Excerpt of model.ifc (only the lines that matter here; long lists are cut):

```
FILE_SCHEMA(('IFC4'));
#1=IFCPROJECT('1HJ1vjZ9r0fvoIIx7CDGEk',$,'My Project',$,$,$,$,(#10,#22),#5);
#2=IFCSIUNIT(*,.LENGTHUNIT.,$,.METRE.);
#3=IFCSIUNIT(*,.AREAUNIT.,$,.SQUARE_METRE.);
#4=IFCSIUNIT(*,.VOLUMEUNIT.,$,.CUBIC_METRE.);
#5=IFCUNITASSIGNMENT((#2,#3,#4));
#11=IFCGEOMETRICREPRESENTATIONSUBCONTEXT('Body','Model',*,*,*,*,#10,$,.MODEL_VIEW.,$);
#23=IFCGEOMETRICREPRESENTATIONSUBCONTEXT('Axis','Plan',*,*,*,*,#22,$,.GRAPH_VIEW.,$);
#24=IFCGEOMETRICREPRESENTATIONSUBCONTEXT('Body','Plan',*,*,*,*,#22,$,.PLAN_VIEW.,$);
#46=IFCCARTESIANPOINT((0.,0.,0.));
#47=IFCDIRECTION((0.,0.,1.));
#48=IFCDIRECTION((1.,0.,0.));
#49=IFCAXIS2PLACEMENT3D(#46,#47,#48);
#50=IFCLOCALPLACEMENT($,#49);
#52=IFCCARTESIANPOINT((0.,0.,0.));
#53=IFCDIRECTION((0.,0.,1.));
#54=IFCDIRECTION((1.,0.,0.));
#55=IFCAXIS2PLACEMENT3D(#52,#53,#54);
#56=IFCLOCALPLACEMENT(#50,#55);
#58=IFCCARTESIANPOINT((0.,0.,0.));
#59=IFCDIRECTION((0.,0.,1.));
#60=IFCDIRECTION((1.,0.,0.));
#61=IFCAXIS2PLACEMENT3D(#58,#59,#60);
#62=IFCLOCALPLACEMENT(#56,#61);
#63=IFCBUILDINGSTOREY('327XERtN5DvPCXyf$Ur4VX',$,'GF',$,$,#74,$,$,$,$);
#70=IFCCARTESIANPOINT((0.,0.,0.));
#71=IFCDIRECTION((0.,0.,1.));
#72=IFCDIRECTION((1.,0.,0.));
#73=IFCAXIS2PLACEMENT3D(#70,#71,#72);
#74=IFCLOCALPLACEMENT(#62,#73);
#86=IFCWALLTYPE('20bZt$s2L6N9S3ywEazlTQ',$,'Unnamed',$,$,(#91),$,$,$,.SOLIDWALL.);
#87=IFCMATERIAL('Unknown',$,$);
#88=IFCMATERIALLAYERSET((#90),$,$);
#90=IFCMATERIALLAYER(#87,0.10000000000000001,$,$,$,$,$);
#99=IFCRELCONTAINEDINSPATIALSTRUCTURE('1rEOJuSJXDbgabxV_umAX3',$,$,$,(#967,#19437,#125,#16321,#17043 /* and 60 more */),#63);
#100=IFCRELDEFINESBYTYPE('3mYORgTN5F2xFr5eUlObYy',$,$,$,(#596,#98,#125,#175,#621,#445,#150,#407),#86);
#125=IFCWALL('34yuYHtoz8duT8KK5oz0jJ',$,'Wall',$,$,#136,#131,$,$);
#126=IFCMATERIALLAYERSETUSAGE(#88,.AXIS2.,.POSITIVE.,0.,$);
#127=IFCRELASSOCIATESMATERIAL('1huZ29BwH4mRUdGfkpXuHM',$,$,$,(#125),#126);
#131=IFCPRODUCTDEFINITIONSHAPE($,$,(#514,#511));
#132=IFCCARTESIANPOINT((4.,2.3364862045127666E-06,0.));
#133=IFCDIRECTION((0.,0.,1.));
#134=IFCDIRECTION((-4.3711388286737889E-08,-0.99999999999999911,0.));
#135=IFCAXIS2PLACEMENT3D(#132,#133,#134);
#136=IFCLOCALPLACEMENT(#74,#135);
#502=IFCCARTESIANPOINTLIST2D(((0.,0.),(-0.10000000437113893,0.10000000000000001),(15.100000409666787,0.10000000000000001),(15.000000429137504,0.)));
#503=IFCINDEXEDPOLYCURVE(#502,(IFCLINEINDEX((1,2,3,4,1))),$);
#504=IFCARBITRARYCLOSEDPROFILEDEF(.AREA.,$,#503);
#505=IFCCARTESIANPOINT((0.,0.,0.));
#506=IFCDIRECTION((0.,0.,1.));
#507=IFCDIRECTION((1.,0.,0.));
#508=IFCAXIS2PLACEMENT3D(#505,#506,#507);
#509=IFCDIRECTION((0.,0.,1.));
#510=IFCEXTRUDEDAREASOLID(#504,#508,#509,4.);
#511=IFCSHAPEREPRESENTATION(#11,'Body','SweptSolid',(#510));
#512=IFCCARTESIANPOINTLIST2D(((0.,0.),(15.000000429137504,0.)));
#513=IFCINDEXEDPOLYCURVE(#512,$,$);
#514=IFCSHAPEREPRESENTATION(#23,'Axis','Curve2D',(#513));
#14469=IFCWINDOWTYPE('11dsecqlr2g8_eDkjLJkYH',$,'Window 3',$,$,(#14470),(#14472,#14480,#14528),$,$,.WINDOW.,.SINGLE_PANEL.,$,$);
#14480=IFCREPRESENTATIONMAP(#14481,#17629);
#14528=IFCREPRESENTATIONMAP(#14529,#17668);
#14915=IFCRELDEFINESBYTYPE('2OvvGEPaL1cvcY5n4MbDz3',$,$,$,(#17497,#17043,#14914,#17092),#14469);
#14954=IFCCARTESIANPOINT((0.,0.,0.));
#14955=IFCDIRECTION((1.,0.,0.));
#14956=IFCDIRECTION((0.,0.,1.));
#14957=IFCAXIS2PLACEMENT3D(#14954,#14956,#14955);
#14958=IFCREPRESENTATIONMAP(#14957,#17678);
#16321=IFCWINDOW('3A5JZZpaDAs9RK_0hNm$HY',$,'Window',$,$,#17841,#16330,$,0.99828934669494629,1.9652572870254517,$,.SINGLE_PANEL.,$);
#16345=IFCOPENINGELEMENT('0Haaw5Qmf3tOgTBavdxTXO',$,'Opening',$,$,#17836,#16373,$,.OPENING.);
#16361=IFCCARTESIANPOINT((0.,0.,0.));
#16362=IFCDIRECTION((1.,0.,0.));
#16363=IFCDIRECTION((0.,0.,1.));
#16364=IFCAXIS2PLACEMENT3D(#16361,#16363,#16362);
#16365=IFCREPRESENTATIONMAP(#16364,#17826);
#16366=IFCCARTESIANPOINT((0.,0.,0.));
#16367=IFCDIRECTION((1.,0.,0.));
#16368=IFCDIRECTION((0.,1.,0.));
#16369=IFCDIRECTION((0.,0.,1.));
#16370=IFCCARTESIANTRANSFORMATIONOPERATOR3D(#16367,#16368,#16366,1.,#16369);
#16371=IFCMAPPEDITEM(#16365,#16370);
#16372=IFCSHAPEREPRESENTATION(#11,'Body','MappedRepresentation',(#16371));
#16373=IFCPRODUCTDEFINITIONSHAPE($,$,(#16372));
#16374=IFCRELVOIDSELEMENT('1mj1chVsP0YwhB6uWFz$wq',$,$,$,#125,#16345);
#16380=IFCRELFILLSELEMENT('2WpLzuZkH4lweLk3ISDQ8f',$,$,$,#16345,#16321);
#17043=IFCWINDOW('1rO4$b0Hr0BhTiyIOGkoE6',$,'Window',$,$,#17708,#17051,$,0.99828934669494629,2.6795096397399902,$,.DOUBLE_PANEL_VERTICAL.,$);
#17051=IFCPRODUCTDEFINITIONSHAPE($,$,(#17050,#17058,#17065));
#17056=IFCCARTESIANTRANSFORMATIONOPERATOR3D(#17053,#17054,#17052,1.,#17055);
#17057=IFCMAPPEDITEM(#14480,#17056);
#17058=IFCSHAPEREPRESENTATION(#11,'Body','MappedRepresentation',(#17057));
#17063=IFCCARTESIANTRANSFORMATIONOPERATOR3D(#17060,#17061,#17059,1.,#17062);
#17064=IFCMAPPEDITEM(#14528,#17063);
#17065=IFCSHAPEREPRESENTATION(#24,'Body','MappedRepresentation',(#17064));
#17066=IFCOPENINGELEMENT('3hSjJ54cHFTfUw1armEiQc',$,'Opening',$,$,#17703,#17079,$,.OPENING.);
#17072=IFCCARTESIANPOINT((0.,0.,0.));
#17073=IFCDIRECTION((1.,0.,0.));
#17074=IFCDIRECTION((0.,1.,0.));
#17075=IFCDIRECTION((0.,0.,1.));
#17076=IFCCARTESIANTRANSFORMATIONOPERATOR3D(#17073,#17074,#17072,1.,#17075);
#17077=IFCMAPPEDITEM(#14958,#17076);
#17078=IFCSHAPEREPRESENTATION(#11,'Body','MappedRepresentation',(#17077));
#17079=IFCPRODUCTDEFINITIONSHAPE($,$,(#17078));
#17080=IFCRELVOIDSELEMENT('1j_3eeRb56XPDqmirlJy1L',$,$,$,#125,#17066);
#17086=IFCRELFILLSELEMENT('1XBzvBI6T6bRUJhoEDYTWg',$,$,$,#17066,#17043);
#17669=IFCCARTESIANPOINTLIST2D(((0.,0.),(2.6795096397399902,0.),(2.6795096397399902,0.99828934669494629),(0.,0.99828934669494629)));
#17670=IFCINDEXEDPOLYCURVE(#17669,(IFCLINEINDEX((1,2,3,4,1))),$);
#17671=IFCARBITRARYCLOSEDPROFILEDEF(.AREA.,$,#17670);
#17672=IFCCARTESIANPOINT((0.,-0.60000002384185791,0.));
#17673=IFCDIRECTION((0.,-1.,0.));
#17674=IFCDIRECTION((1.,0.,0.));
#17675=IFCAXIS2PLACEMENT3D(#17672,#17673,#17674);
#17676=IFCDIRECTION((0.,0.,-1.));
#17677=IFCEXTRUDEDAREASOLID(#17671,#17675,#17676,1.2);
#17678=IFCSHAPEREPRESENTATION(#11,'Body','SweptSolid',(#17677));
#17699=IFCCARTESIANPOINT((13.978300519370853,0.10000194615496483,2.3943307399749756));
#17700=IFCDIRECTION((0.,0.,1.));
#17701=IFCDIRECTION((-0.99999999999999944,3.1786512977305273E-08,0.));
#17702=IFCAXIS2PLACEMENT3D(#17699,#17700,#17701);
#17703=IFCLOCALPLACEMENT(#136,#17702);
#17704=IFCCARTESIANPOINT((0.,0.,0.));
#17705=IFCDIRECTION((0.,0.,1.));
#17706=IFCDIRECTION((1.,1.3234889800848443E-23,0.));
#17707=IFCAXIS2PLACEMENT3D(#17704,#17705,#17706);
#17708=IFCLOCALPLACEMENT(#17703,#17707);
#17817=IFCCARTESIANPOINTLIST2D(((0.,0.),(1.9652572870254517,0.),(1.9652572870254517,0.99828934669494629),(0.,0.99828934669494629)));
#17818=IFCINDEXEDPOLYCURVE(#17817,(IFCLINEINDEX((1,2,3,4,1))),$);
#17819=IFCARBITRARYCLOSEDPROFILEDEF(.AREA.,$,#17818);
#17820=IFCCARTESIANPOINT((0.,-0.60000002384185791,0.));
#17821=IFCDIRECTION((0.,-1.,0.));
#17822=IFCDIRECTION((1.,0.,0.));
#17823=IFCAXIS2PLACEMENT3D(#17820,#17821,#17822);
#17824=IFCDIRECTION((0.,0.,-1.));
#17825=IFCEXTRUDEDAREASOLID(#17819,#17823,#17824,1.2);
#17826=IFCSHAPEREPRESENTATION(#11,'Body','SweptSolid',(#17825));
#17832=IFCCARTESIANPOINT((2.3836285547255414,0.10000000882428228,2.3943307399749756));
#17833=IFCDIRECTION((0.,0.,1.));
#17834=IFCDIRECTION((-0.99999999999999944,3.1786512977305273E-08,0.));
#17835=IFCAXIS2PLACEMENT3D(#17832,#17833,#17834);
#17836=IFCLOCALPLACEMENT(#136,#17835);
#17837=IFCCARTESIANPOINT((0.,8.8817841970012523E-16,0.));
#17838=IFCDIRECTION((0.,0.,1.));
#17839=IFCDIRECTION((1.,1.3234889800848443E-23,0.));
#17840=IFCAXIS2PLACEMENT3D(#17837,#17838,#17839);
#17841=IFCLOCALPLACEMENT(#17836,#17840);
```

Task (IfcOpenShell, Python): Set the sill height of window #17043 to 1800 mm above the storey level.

```python
import numpy as np
import ifcopenshell
import ifcopenshell.api.geometry
import ifcopenshell.geom
import ifcopenshell.util.element
import ifcopenshell.util.placement
import ifcopenshell.util.shape
import ifcopenshell.util.unit

model = ifcopenshell.open("model.ifc")
unit_scale = ifcopenshell.util.unit.calculate_unit_scale(model)

window = model.by_guid("1rO4$b0Hr0BhTiyIOGkoE6")
opening = window.FillsVoids[0].RelatingOpeningElement
storey = ifcopenshell.util.element.get_container(window, ifc_class="IfcBuildingStorey")
level = ifcopenshell.util.placement.get_local_placement(storey.ObjectPlacement)[2, 3]

# The opening's origin need not be at the sill, so measure its lowest point.
shape = ifcopenshell.geom.create_shape(ifcopenshell.geom.settings(), opening)
bottom = ifcopenshell.util.shape.get_shape_bottom_elevation(shape, shape.geometry) / unit_scale
dz = level + 1.8 - bottom

shift = np.array([0.0, 0.0, dz])
# The window is placed relative to its opening, so it follows when the opening moves.
matrix = ifcopenshell.util.placement.get_local_placement(opening.ObjectPlacement)
matrix[:3, 3] += shift
ifcopenshell.api.geometry.edit_object_placement(
    model, product=opening, matrix=matrix, is_si=False, should_transform_children=True
)

print(f"moved by {dz * unit_scale:+.3f} m")

model.write("model_v2.ifc")
```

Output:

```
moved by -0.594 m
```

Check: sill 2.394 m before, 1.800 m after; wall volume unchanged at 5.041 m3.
